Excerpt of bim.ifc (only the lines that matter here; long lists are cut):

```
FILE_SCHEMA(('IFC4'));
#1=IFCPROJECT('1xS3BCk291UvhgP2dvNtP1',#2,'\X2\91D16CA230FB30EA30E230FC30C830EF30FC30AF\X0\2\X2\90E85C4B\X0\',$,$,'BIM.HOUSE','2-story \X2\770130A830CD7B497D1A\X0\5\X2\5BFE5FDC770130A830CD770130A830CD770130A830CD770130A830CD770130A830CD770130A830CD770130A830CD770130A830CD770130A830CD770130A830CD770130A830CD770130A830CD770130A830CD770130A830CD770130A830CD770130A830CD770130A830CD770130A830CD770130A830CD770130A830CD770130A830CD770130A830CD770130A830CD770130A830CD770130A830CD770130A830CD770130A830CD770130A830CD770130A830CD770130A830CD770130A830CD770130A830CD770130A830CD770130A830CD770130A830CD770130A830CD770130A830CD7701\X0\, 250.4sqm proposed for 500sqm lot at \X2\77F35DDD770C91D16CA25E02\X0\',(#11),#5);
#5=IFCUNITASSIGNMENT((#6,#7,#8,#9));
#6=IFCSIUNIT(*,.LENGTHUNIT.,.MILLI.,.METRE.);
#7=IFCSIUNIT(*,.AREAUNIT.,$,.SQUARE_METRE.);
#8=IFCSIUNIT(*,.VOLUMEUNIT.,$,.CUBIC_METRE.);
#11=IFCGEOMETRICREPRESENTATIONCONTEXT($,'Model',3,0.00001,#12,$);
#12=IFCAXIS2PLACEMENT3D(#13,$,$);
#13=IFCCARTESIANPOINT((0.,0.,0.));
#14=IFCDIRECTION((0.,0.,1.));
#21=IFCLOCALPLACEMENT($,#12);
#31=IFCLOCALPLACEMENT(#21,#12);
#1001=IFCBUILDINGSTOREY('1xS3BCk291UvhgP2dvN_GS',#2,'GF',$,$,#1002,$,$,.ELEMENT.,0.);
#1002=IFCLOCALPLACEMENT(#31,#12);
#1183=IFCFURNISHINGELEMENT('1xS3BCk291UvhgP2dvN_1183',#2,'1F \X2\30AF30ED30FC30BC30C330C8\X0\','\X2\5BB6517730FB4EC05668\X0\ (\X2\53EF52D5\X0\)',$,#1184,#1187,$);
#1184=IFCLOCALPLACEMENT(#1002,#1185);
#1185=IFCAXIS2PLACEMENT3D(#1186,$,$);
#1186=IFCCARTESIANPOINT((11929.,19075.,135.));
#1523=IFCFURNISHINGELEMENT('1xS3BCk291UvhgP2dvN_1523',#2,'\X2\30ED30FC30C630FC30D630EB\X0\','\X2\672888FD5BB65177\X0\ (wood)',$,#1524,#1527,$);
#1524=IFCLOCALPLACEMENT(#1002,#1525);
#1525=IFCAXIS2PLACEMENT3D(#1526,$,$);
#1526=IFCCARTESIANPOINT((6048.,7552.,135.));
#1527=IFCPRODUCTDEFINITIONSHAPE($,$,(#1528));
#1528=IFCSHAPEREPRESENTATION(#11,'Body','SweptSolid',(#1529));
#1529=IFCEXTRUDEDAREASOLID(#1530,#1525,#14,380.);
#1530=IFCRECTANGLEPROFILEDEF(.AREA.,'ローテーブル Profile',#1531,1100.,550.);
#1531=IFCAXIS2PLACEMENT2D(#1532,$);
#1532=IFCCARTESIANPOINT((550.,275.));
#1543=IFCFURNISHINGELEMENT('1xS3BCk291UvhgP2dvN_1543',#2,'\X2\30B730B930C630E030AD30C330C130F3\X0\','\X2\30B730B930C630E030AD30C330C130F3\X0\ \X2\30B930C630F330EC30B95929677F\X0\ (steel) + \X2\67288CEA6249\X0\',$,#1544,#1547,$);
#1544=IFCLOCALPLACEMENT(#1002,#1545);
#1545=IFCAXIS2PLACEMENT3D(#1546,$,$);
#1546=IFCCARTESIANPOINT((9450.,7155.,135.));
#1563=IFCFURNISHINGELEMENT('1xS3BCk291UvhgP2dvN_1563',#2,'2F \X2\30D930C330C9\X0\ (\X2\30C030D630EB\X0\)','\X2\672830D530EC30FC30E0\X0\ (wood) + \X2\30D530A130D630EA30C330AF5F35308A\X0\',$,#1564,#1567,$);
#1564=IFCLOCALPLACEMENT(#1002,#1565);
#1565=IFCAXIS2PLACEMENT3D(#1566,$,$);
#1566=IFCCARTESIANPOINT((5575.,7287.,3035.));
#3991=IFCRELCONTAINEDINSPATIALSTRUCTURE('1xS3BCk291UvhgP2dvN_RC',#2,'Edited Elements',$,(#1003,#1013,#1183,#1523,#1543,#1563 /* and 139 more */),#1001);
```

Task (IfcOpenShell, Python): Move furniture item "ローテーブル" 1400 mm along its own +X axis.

```python
import ifcopenshell
import ifcopenshell.api.geometry
import ifcopenshell.util.placement

model = ifcopenshell.open("bim.ifc")

item = model.by_guid("1xS3BCk291UvhgP2dvN_1523")
matrix = ifcopenshell.util.placement.get_local_placement(item.ObjectPlacement)
matrix[:3, 3] += matrix[:3, 0] * 1400.0
ifcopenshell.api.geometry.edit_object_placement(model, product=item, matrix=matrix, is_si=False)

print(ifcopenshell.util.placement.get_local_placement(item.ObjectPlacement).round(3) + 0.0)

model.write("bim_rev.ifc")
```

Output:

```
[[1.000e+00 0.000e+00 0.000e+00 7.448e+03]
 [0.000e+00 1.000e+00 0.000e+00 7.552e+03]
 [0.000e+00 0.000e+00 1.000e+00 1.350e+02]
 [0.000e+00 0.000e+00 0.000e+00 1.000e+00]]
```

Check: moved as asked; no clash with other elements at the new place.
